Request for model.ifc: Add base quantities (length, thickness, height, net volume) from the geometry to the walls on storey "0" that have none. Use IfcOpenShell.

First a look at what the model holds.

```python
import ifcopenshell
import ifcopenshell.util.element
import ifcopenshell.util.unit

model = ifcopenshell.open("model.ifc")
print(model.schema)
for unit_type in ("LENGTHUNIT", "AREAUNIT", "VOLUMEUNIT"):
    print(unit_type, ifcopenshell.util.unit.calculate_unit_scale(model, unit_type))
storey = next(s for s in model.by_type("IfcBuildingStorey") if s.Name == "0")
walls = [e for e in ifcopenshell.util.element.get_decomposition(storey) if e.is_a("IfcWall")]
for e in sorted(walls, key=lambda e: e.id()):
    print(e.id(), e.is_a(), e.Name, list(ifcopenshell.util.element.get_psets(e, qtos_only=True)), sep=" | ")
```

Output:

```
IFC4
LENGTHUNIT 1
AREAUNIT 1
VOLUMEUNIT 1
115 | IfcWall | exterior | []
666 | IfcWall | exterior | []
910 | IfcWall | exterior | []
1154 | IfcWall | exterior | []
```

```python
import ifcopenshell
import ifcopenshell.api.pset
import ifcopenshell.geom
import ifcopenshell.util.element
import ifcopenshell.util.shape
import ifcopenshell.util.unit

model = ifcopenshell.open("model.ifc")
unit_scale = ifcopenshell.util.unit.calculate_unit_scale(model)
volume_scale = ifcopenshell.util.unit.calculate_unit_scale(model, "VOLUMEUNIT")
settings = ifcopenshell.geom.settings()

storey = next(s for s in model.by_type("IfcBuildingStorey") if s.Name == "0")
walls = [e for e in ifcopenshell.util.element.get_decomposition(storey) if e.is_a("IfcWall")]

for e in sorted(walls, key=lambda e: e.id()):
    if ifcopenshell.util.element.get_psets(e, qtos_only=True, should_inherit=False):
        continue
    # Geometry comes back in metres, in the element's own axes.
    shape = ifcopenshell.geom.create_shape(settings, e)
    values = {
        "Length": ifcopenshell.util.shape.get_x(shape.geometry) / unit_scale,
        "Width": ifcopenshell.util.shape.get_y(shape.geometry) / unit_scale,
        "Height": ifcopenshell.util.shape.get_z(shape.geometry) / unit_scale,
        "NetVolume": ifcopenshell.util.shape.get_volume(shape.geometry) / volume_scale,
    }
    qto = ifcopenshell.api.pset.add_qto(model, product=e, name="Qto_WallBaseQuantities")
    ifcopenshell.api.pset.edit_qto(model, qto=qto, properties=values)
    print(e.id(), {k: round(v, 3) for k, v in values.items()})

model.write("model-out.ifc")
```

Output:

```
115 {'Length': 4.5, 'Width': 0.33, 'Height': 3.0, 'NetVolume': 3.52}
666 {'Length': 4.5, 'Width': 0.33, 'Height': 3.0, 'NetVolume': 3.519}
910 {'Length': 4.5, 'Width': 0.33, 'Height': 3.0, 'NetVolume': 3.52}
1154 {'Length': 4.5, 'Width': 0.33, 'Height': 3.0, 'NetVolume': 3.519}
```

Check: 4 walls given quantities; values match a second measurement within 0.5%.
